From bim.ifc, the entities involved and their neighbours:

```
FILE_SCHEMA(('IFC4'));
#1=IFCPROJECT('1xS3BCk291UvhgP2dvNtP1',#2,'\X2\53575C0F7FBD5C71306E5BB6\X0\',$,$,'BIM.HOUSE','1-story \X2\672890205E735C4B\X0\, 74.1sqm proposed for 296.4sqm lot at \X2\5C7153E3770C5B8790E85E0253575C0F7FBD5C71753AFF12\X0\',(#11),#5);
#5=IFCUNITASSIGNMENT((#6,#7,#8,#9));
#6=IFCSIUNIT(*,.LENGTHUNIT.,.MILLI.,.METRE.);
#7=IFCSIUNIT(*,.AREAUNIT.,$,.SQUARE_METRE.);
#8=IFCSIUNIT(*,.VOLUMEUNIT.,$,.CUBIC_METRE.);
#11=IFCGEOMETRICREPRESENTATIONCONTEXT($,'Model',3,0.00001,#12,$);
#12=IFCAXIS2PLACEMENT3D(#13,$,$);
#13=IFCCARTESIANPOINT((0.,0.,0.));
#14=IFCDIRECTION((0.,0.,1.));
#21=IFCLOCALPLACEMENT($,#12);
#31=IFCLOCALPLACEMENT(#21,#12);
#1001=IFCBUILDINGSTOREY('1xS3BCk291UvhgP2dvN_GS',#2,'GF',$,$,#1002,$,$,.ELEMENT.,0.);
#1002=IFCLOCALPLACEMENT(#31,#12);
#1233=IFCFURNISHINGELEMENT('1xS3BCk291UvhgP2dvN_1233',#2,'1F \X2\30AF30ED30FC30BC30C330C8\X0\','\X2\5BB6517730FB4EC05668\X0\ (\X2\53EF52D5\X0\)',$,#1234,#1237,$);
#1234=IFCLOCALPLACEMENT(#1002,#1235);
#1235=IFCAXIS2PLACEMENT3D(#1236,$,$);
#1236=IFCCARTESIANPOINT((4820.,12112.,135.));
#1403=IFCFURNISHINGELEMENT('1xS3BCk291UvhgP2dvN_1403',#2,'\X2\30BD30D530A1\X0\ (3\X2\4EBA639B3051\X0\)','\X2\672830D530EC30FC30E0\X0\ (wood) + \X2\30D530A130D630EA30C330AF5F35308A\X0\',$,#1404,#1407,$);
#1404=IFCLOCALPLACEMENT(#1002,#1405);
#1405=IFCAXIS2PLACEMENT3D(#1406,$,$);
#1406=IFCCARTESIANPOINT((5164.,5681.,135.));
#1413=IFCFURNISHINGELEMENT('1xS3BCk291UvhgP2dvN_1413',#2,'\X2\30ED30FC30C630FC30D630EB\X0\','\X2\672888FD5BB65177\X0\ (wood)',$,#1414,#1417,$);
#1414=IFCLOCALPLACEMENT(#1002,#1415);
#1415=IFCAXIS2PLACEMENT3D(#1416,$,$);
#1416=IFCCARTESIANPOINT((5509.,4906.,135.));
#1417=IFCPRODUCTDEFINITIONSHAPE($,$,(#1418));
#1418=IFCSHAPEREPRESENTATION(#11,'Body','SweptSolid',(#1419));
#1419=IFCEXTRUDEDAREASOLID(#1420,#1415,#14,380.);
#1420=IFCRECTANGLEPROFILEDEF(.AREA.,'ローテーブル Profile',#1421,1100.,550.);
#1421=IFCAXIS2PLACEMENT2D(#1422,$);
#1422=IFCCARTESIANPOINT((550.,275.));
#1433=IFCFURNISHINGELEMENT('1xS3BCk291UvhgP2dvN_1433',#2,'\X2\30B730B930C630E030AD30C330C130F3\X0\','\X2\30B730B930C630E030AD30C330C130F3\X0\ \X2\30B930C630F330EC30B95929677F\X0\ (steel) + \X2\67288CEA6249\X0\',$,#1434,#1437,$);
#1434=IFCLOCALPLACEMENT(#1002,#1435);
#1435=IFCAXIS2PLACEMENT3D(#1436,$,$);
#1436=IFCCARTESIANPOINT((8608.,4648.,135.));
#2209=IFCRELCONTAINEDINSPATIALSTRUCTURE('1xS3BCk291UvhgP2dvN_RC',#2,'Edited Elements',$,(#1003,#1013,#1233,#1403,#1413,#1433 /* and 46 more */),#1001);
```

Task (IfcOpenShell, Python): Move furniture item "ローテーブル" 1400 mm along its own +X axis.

```python
import ifcopenshell
import ifcopenshell.api.geometry
import ifcopenshell.util.placement
import ifcopenshell.util.unit

model = ifcopenshell.open("bim.ifc")
unit_scale = ifcopenshell.util.unit.calculate_unit_scale(model)

item = model.by_guid("1xS3BCk291UvhgP2dvN_1413")
matrix = ifcopenshell.util.placement.get_local_placement(item.ObjectPlacement)
matrix[:3, 3] += matrix[:3, 0] * 1.4 / unit_scale
ifcopenshell.api.geometry.edit_object_placement(model, product=item, matrix=matrix, is_si=False)

print(ifcopenshell.util.placement.get_local_placement(item.ObjectPlacement).round(3) + 0.0)

model.write("bim_edited.ifc")
```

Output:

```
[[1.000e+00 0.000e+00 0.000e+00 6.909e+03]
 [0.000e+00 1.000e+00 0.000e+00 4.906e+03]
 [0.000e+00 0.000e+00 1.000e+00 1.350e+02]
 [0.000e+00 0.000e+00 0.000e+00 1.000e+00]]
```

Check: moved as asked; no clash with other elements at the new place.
